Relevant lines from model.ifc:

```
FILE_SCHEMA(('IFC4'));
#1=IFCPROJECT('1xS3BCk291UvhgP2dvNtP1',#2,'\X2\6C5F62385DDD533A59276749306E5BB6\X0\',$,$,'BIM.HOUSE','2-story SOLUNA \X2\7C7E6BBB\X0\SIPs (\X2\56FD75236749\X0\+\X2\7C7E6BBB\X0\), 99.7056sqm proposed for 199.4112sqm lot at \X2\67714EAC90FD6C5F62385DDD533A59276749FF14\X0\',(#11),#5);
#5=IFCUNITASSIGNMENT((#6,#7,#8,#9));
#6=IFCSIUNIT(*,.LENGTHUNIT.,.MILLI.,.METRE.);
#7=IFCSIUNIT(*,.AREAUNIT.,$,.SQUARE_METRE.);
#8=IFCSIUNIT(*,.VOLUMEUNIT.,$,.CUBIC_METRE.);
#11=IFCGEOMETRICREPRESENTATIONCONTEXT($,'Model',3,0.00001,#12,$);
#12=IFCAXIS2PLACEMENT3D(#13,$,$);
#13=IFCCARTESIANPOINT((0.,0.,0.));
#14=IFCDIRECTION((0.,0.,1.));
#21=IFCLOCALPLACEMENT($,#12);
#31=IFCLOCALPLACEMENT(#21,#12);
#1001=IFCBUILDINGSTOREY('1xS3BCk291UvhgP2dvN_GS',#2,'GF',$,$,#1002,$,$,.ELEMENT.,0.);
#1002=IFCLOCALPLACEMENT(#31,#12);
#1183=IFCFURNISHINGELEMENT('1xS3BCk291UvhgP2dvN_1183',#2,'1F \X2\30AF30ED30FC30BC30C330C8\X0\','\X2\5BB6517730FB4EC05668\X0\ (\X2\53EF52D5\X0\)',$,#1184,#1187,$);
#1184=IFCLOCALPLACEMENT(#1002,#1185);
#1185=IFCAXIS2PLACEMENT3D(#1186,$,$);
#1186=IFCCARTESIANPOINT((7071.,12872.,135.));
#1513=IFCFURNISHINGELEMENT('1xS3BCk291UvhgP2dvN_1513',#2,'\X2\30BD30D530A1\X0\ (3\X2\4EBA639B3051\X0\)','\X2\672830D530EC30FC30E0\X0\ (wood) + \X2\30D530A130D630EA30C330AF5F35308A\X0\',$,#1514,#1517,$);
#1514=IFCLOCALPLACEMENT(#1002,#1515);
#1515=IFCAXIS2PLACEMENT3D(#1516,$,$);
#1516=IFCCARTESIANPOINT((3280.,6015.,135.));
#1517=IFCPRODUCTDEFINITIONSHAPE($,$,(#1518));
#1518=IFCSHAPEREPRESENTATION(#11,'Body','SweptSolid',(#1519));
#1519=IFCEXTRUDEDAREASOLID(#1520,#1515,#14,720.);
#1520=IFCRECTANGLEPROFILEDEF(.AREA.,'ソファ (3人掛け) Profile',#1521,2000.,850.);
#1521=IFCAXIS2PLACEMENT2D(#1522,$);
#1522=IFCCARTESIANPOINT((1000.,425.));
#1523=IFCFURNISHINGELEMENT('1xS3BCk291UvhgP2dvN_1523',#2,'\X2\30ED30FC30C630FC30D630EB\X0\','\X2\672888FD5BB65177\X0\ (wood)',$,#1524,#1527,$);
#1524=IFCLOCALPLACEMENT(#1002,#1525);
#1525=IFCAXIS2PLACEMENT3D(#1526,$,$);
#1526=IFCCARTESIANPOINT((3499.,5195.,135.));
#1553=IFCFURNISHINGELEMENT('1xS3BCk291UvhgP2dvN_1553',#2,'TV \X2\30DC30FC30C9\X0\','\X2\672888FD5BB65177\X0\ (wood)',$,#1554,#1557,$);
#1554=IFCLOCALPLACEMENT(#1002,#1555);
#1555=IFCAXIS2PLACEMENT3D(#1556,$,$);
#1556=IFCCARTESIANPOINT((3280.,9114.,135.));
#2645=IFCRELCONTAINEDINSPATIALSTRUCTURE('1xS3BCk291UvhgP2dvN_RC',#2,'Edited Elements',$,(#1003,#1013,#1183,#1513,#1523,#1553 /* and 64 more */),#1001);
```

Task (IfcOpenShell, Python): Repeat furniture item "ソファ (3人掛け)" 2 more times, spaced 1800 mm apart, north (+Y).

```python
import numpy as np
import ifcopenshell
import ifcopenshell.api.geometry
import ifcopenshell.api.root
import ifcopenshell.util.element
import ifcopenshell.util.placement
import ifcopenshell.util.unit

model = ifcopenshell.open("model.ifc")
unit_scale = ifcopenshell.util.unit.calculate_unit_scale(model)


def reuse_history(source, copy):
    """copy_class also copies each property set's owner history, people and application; keep the originals."""
    for rel in copy.IsDefinedBy:
        if rel.is_a("IfcRelDefinesByProperties") and (history := rel.RelatingPropertyDefinition.OwnerHistory):
            rel.RelatingPropertyDefinition.OwnerHistory = source.OwnerHistory
            ifcopenshell.util.element.remove_deep2(model, history)


source = model.by_guid("1xS3BCk291UvhgP2dvN_1513")
base = ifcopenshell.util.placement.get_local_placement(source.ObjectPlacement)
step = np.array([0.0, 1.0, 0.0]) * 1.8 / unit_scale

for i in range(1, 3):
    copy = ifcopenshell.api.root.copy_class(model, product=source)
    copy.Representation = ifcopenshell.util.element.copy_deep(
        model, source.Representation, exclude=["IfcGeometricRepresentationContext", "IfcRepresentationMap"]
    )
    reuse_history(source, copy)
    matrix = base.copy()
    matrix[:3, 3] += i * step
    print("added at", matrix[:3, 3].round(3) + 0.0)
    ifcopenshell.api.geometry.edit_object_placement(model, product=copy, matrix=matrix, is_si=False)

model.write("model_rev.ifc")
```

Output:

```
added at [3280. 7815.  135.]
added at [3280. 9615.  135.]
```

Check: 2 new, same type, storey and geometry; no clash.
